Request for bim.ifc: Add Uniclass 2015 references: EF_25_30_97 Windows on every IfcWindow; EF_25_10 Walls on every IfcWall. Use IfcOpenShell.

First a look at what the model holds.

```python
import ifcopenshell

model = ifcopenshell.open("bim.ifc")
print(model.schema)
print("classifications:", [c.Name for c in model.by_type("IfcClassification")])
for ifc_class in ("IfcDoor", "IfcRoof", "IfcStair", "IfcWall", "IfcWindow"):
    print(ifc_class, len(model.by_type(ifc_class)))
```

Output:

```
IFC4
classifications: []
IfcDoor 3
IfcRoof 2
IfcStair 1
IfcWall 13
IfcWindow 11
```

```python
import ifcopenshell
import ifcopenshell.api.classification

model = ifcopenshell.open("bim.ifc")

system = ifcopenshell.api.classification.add_classification(model, classification="Uniclass 2015")

codes = {
    "IfcWindow": ("EF_25_30_97", "Windows"),
    "IfcWall": ("EF_25_10", "Walls"),
}
for ifc_class, (code, name) in codes.items():
    products = model.by_type(ifc_class)
    ifcopenshell.api.classification.add_reference(
        model, products=products, classification=system, identification=code, name=name
    )
    print(code, len(products))

model.write("bim-out.ifc")
```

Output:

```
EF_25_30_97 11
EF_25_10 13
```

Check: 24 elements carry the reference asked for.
